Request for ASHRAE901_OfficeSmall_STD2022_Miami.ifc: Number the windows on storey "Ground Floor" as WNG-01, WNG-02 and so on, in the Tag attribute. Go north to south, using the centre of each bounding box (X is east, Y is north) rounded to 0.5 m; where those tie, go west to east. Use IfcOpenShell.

First a look at what the model holds.

```python
import ifcopenshell
import ifcopenshell.util.element
import ifcopenshell.util.placement

model = ifcopenshell.open("ASHRAE901_OfficeSmall_STD2022_Miami.ifc")
print(model.schema)
storey = next(s for s in model.by_type("IfcBuildingStorey") if s.Name == "Ground Floor")
windows = [e for e in ifcopenshell.util.element.get_decomposition(storey) if e.is_a("IfcWindow")]
for e in sorted(windows, key=lambda e: e.id()):
    origin = ifcopenshell.util.placement.get_local_placement(e.ObjectPlacement)[:3, 3]
    print(e.id(), e.Tag, e.Name, origin.round(2) + 0.0, sep=" | ")
```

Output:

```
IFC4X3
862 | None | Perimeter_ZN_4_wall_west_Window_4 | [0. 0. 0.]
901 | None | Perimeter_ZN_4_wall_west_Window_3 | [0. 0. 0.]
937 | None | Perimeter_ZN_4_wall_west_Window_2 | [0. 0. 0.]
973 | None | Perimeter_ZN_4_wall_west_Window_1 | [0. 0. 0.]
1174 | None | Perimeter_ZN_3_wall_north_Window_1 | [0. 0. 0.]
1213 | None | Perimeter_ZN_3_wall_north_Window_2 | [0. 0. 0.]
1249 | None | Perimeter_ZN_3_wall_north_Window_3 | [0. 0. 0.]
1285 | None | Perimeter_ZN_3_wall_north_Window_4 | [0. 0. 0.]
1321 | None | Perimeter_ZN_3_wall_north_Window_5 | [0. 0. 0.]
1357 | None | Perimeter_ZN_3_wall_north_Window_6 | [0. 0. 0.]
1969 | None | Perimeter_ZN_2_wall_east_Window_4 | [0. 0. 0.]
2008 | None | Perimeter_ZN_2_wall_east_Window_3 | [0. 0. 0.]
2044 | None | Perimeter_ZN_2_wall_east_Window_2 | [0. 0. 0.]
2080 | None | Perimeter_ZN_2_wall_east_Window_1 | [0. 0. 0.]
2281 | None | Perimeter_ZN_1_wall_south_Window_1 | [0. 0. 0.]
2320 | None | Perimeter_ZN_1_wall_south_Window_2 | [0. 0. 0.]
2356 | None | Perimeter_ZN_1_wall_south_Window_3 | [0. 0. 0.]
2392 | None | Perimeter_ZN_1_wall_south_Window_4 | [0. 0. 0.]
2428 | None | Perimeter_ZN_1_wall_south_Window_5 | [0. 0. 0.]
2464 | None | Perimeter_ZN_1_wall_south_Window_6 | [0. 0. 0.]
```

```python
import ifcopenshell
import ifcopenshell.geom
import ifcopenshell.util.element
import ifcopenshell.util.shape

model = ifcopenshell.open("ASHRAE901_OfficeSmall_STD2022_Miami.ifc")
settings = ifcopenshell.geom.settings()
settings.set("use-world-coords", True)


def centre(element):
    shape = ifcopenshell.geom.create_shape(settings, element)
    return ifcopenshell.util.shape.get_bbox_centroid(shape.geometry)


storey = next(s for s in model.by_type("IfcBuildingStorey") if s.Name == "Ground Floor")
windows = [e for e in ifcopenshell.util.element.get_decomposition(storey) if e.is_a("IfcWindow")]

# Insertion points can sit at a corner or the storey origin, so sort by the geometry (in metres).
centres = {e: centre(e) for e in windows}
windows.sort(key=lambda e: (-round(centres[e][1] / 0.5), centres[e][0]))

for i, e in enumerate(windows, start=1):
    number = f"WNG-{i:02d}"
    e.Tag = number
    print(e.id(), number)

model.write("ASHRAE901_OfficeSmall_STD2022_Miami_v2.ifc")
```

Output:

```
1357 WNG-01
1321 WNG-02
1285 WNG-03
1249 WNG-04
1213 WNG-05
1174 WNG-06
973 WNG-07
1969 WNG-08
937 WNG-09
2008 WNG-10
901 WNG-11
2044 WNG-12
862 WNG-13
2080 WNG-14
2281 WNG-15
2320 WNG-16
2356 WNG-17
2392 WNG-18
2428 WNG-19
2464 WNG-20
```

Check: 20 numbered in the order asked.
